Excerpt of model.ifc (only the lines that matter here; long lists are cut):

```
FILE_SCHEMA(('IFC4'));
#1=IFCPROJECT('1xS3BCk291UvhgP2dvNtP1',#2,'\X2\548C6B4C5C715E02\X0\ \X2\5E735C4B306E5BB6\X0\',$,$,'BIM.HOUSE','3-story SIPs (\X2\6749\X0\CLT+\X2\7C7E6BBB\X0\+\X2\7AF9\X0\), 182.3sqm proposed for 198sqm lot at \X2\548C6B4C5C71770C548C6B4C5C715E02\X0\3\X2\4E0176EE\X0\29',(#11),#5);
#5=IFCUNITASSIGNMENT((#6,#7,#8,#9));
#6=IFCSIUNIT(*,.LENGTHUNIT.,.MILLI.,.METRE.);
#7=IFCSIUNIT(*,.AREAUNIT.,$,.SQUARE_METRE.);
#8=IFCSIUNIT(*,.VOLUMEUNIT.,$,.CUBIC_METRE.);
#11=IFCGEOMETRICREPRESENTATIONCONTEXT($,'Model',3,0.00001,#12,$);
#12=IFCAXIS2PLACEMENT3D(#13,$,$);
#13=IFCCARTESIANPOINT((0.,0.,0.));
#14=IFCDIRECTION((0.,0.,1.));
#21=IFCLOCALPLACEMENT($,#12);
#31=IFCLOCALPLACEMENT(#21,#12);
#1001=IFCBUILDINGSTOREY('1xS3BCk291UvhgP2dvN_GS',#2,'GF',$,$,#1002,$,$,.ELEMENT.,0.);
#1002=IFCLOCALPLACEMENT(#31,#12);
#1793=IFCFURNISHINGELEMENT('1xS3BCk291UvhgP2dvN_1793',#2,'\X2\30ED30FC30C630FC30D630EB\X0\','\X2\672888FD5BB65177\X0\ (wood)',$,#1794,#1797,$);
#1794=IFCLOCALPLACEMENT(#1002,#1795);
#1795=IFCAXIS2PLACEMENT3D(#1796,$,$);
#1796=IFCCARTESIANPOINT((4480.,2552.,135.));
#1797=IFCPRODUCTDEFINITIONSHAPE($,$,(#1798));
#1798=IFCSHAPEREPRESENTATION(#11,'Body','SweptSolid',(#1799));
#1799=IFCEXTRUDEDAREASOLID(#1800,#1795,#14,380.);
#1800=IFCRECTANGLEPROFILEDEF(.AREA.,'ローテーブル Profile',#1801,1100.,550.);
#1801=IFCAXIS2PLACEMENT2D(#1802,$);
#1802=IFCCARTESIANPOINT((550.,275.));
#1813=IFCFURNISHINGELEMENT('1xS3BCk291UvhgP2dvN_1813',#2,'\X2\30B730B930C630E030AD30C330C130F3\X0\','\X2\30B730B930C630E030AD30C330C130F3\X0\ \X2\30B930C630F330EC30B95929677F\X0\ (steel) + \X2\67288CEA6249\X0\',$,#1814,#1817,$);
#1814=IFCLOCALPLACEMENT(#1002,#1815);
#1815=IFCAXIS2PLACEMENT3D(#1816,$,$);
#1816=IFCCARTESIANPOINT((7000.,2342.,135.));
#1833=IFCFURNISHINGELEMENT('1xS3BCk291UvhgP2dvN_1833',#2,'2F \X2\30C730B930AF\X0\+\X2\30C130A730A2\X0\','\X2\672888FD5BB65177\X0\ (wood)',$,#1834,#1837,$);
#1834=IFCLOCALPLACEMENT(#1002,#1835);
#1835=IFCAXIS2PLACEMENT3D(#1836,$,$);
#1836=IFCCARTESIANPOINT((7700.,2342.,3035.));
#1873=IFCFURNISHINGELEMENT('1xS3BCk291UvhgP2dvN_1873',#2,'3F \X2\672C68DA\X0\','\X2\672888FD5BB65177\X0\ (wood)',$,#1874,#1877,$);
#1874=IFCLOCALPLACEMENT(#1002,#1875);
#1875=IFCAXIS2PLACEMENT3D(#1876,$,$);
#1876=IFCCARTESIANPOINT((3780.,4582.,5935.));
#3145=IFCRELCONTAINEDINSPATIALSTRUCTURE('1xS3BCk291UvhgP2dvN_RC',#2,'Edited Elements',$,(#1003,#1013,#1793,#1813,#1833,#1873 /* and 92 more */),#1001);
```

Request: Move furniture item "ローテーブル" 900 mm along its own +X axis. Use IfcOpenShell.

```python
import ifcopenshell
import ifcopenshell.api.geometry
import ifcopenshell.util.placement

model = ifcopenshell.open("model.ifc")

item = model.by_guid("1xS3BCk291UvhgP2dvN_1793")
matrix = ifcopenshell.util.placement.get_local_placement(item.ObjectPlacement)
matrix[:3, 3] += matrix[:3, 0] * 900.0
ifcopenshell.api.geometry.edit_object_placement(model, product=item, matrix=matrix, is_si=False)

print(ifcopenshell.util.placement.get_local_placement(item.ObjectPlacement).round(3) + 0.0)

model.write("model_v2.ifc")
```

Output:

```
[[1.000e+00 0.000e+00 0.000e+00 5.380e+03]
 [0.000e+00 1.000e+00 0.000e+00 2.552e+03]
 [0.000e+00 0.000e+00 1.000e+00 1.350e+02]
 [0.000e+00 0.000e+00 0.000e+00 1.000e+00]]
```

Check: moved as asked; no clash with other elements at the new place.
